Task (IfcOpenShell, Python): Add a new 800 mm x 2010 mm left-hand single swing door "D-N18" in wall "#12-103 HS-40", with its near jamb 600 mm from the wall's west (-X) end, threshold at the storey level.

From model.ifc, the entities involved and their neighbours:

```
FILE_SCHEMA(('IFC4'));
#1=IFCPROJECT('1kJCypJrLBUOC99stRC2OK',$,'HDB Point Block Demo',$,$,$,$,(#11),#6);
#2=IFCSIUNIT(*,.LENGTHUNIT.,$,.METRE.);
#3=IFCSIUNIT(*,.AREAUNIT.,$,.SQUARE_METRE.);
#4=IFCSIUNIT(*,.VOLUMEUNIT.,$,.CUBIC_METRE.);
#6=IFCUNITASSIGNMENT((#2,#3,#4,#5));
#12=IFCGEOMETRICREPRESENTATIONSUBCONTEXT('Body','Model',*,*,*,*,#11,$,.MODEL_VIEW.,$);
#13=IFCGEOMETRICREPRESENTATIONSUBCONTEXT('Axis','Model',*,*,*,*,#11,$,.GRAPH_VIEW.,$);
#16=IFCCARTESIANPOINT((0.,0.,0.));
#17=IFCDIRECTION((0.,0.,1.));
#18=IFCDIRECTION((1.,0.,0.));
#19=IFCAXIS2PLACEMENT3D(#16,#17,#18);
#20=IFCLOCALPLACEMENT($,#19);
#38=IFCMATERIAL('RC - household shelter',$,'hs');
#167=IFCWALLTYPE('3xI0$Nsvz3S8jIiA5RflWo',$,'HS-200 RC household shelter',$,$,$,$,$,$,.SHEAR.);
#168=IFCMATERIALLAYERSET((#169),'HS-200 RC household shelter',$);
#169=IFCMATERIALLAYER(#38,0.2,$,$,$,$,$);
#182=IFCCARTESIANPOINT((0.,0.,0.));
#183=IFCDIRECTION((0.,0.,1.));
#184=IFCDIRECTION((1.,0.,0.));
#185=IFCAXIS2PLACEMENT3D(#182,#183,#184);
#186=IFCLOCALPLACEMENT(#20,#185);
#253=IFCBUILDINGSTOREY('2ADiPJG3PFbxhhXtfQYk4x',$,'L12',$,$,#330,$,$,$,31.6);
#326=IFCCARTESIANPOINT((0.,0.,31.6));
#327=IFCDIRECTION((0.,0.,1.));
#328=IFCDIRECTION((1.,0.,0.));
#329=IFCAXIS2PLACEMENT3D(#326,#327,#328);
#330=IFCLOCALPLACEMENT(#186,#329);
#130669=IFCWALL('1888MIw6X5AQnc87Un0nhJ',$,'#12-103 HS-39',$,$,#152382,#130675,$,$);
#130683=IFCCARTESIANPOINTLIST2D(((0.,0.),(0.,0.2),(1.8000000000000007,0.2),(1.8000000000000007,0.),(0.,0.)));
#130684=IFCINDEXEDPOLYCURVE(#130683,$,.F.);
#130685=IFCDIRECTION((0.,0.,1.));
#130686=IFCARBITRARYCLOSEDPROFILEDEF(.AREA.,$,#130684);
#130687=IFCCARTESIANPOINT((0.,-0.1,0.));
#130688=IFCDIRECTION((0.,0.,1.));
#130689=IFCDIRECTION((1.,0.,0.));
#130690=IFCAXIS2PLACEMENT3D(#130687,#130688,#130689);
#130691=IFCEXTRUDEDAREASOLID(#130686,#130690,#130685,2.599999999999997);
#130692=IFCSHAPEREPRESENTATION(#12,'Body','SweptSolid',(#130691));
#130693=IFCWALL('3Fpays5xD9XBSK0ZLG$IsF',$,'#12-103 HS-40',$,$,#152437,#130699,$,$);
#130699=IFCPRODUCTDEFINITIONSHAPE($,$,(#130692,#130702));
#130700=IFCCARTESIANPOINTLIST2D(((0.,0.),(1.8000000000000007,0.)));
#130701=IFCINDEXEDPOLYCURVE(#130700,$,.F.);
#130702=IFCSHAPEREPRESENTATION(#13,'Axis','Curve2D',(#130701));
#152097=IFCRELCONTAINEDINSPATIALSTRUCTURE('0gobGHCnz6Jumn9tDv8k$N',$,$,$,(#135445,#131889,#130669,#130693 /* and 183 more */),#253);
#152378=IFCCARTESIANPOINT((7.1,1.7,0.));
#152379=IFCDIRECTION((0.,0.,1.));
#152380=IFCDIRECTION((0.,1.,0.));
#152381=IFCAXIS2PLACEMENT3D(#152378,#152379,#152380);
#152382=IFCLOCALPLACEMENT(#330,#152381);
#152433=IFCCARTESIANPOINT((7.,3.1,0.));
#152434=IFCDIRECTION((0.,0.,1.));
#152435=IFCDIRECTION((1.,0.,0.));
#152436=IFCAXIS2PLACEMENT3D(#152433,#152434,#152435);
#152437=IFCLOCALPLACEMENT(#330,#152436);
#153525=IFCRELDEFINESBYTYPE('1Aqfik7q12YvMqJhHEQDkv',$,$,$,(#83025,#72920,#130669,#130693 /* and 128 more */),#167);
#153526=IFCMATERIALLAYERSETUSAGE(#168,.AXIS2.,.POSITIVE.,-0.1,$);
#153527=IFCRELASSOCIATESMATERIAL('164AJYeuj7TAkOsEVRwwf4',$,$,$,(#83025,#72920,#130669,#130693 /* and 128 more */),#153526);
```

```python
import numpy as np
import ifcopenshell
import ifcopenshell.api.feature
import ifcopenshell.api.geometry
import ifcopenshell.api.root
import ifcopenshell.api.spatial
import ifcopenshell.geom
import ifcopenshell.util.element
import ifcopenshell.util.placement
import ifcopenshell.util.representation
import ifcopenshell.util.shape
import ifcopenshell.util.unit

model = ifcopenshell.open("model.ifc")
unit_scale = ifcopenshell.util.unit.calculate_unit_scale(model)
settings = ifcopenshell.geom.settings()


def volume(element):
    """Net volume in cubic metres, openings subtracted."""
    shape = ifcopenshell.geom.create_shape(settings, element)
    return ifcopenshell.util.shape.get_volume(shape.geometry)


wall = model.by_guid("3Fpays5xD9XBSK0ZLG$IsF")
storey = ifcopenshell.util.element.get_container(wall, ifc_class="IfcBuildingStorey")
context = ifcopenshell.util.representation.get_context(model, "Model", "Body", "MODEL_VIEW")
before = volume(wall)

width, height, from_end, sill = 0.8, 2.01, 0.6, 0.0  # metres

# The wall runs along its own X axis, and the end named is its -X end.
wall_shape = ifcopenshell.geom.create_shape(settings, wall)
x, y, z = ifcopenshell.util.shape.get_vertices(wall_shape.geometry).T
start = x.min() + from_end
face, thickness = float(y.min()), float(y.max() - y.min())
wall_matrix = ifcopenshell.util.placement.get_local_placement(wall.ObjectPlacement)
level = ifcopenshell.util.placement.get_local_placement(storey.ObjectPlacement)[2, 3]


def in_wall(x, y):
    """Placement at x, y metres in the wall's axes, at sill height."""
    matrix = wall_matrix.copy()
    matrix[:, 3] = wall_matrix @ np.array([x / unit_scale, y / unit_scale, 0.0, 1.0])
    matrix[2, 3] = level + sill / unit_scale
    return matrix


# Opening: a box that overshoots both wall faces by 50 mm.
opening = ifcopenshell.api.root.create_entity(model, ifc_class="IfcOpeningElement", predefined_type="OPENING")
box = ifcopenshell.api.geometry.add_wall_representation(
    model, context=context, length=width, height=height, thickness=thickness + 0.1
)
ifcopenshell.api.geometry.assign_representation(model, product=opening, representation=box)
ifcopenshell.api.geometry.edit_object_placement(model, product=opening, matrix=in_wall(start, face - 0.05), is_si=False)
ifcopenshell.api.feature.add_feature(model, feature=opening, element=wall)

door = ifcopenshell.api.root.create_entity(model, ifc_class="IfcDoor", name="D-N18", predefined_type="DOOR")
door.OverallWidth, door.OverallHeight = width / unit_scale, height / unit_scale
door.OperationType = "SINGLE_SWING_LEFT"
body = ifcopenshell.api.geometry.add_door_representation(
    model,
    context=context,
    overall_width=door.OverallWidth,
    overall_height=door.OverallHeight,
    operation_type="SINGLE_SWING_LEFT",
    lining_properties={"LiningDepth": thickness / unit_scale, "ThresholdDepth": thickness / unit_scale},
)
ifcopenshell.api.geometry.assign_representation(model, product=door, representation=body)
ifcopenshell.api.spatial.assign_container(model, products=[door], relating_structure=storey)
ifcopenshell.api.feature.add_filling(model, opening=opening, element=door)

# The lining spans the wall, so the door starts at the wall face.
ifcopenshell.api.geometry.edit_object_placement(model, product=door, matrix=in_wall(start, face), is_si=False)

after = volume(wall)

print(f"wall volume {before:.3f} -> {after:.3f} m3")

model.write("model_edited.ifc")
```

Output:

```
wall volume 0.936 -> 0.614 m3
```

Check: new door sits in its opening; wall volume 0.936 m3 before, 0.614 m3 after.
